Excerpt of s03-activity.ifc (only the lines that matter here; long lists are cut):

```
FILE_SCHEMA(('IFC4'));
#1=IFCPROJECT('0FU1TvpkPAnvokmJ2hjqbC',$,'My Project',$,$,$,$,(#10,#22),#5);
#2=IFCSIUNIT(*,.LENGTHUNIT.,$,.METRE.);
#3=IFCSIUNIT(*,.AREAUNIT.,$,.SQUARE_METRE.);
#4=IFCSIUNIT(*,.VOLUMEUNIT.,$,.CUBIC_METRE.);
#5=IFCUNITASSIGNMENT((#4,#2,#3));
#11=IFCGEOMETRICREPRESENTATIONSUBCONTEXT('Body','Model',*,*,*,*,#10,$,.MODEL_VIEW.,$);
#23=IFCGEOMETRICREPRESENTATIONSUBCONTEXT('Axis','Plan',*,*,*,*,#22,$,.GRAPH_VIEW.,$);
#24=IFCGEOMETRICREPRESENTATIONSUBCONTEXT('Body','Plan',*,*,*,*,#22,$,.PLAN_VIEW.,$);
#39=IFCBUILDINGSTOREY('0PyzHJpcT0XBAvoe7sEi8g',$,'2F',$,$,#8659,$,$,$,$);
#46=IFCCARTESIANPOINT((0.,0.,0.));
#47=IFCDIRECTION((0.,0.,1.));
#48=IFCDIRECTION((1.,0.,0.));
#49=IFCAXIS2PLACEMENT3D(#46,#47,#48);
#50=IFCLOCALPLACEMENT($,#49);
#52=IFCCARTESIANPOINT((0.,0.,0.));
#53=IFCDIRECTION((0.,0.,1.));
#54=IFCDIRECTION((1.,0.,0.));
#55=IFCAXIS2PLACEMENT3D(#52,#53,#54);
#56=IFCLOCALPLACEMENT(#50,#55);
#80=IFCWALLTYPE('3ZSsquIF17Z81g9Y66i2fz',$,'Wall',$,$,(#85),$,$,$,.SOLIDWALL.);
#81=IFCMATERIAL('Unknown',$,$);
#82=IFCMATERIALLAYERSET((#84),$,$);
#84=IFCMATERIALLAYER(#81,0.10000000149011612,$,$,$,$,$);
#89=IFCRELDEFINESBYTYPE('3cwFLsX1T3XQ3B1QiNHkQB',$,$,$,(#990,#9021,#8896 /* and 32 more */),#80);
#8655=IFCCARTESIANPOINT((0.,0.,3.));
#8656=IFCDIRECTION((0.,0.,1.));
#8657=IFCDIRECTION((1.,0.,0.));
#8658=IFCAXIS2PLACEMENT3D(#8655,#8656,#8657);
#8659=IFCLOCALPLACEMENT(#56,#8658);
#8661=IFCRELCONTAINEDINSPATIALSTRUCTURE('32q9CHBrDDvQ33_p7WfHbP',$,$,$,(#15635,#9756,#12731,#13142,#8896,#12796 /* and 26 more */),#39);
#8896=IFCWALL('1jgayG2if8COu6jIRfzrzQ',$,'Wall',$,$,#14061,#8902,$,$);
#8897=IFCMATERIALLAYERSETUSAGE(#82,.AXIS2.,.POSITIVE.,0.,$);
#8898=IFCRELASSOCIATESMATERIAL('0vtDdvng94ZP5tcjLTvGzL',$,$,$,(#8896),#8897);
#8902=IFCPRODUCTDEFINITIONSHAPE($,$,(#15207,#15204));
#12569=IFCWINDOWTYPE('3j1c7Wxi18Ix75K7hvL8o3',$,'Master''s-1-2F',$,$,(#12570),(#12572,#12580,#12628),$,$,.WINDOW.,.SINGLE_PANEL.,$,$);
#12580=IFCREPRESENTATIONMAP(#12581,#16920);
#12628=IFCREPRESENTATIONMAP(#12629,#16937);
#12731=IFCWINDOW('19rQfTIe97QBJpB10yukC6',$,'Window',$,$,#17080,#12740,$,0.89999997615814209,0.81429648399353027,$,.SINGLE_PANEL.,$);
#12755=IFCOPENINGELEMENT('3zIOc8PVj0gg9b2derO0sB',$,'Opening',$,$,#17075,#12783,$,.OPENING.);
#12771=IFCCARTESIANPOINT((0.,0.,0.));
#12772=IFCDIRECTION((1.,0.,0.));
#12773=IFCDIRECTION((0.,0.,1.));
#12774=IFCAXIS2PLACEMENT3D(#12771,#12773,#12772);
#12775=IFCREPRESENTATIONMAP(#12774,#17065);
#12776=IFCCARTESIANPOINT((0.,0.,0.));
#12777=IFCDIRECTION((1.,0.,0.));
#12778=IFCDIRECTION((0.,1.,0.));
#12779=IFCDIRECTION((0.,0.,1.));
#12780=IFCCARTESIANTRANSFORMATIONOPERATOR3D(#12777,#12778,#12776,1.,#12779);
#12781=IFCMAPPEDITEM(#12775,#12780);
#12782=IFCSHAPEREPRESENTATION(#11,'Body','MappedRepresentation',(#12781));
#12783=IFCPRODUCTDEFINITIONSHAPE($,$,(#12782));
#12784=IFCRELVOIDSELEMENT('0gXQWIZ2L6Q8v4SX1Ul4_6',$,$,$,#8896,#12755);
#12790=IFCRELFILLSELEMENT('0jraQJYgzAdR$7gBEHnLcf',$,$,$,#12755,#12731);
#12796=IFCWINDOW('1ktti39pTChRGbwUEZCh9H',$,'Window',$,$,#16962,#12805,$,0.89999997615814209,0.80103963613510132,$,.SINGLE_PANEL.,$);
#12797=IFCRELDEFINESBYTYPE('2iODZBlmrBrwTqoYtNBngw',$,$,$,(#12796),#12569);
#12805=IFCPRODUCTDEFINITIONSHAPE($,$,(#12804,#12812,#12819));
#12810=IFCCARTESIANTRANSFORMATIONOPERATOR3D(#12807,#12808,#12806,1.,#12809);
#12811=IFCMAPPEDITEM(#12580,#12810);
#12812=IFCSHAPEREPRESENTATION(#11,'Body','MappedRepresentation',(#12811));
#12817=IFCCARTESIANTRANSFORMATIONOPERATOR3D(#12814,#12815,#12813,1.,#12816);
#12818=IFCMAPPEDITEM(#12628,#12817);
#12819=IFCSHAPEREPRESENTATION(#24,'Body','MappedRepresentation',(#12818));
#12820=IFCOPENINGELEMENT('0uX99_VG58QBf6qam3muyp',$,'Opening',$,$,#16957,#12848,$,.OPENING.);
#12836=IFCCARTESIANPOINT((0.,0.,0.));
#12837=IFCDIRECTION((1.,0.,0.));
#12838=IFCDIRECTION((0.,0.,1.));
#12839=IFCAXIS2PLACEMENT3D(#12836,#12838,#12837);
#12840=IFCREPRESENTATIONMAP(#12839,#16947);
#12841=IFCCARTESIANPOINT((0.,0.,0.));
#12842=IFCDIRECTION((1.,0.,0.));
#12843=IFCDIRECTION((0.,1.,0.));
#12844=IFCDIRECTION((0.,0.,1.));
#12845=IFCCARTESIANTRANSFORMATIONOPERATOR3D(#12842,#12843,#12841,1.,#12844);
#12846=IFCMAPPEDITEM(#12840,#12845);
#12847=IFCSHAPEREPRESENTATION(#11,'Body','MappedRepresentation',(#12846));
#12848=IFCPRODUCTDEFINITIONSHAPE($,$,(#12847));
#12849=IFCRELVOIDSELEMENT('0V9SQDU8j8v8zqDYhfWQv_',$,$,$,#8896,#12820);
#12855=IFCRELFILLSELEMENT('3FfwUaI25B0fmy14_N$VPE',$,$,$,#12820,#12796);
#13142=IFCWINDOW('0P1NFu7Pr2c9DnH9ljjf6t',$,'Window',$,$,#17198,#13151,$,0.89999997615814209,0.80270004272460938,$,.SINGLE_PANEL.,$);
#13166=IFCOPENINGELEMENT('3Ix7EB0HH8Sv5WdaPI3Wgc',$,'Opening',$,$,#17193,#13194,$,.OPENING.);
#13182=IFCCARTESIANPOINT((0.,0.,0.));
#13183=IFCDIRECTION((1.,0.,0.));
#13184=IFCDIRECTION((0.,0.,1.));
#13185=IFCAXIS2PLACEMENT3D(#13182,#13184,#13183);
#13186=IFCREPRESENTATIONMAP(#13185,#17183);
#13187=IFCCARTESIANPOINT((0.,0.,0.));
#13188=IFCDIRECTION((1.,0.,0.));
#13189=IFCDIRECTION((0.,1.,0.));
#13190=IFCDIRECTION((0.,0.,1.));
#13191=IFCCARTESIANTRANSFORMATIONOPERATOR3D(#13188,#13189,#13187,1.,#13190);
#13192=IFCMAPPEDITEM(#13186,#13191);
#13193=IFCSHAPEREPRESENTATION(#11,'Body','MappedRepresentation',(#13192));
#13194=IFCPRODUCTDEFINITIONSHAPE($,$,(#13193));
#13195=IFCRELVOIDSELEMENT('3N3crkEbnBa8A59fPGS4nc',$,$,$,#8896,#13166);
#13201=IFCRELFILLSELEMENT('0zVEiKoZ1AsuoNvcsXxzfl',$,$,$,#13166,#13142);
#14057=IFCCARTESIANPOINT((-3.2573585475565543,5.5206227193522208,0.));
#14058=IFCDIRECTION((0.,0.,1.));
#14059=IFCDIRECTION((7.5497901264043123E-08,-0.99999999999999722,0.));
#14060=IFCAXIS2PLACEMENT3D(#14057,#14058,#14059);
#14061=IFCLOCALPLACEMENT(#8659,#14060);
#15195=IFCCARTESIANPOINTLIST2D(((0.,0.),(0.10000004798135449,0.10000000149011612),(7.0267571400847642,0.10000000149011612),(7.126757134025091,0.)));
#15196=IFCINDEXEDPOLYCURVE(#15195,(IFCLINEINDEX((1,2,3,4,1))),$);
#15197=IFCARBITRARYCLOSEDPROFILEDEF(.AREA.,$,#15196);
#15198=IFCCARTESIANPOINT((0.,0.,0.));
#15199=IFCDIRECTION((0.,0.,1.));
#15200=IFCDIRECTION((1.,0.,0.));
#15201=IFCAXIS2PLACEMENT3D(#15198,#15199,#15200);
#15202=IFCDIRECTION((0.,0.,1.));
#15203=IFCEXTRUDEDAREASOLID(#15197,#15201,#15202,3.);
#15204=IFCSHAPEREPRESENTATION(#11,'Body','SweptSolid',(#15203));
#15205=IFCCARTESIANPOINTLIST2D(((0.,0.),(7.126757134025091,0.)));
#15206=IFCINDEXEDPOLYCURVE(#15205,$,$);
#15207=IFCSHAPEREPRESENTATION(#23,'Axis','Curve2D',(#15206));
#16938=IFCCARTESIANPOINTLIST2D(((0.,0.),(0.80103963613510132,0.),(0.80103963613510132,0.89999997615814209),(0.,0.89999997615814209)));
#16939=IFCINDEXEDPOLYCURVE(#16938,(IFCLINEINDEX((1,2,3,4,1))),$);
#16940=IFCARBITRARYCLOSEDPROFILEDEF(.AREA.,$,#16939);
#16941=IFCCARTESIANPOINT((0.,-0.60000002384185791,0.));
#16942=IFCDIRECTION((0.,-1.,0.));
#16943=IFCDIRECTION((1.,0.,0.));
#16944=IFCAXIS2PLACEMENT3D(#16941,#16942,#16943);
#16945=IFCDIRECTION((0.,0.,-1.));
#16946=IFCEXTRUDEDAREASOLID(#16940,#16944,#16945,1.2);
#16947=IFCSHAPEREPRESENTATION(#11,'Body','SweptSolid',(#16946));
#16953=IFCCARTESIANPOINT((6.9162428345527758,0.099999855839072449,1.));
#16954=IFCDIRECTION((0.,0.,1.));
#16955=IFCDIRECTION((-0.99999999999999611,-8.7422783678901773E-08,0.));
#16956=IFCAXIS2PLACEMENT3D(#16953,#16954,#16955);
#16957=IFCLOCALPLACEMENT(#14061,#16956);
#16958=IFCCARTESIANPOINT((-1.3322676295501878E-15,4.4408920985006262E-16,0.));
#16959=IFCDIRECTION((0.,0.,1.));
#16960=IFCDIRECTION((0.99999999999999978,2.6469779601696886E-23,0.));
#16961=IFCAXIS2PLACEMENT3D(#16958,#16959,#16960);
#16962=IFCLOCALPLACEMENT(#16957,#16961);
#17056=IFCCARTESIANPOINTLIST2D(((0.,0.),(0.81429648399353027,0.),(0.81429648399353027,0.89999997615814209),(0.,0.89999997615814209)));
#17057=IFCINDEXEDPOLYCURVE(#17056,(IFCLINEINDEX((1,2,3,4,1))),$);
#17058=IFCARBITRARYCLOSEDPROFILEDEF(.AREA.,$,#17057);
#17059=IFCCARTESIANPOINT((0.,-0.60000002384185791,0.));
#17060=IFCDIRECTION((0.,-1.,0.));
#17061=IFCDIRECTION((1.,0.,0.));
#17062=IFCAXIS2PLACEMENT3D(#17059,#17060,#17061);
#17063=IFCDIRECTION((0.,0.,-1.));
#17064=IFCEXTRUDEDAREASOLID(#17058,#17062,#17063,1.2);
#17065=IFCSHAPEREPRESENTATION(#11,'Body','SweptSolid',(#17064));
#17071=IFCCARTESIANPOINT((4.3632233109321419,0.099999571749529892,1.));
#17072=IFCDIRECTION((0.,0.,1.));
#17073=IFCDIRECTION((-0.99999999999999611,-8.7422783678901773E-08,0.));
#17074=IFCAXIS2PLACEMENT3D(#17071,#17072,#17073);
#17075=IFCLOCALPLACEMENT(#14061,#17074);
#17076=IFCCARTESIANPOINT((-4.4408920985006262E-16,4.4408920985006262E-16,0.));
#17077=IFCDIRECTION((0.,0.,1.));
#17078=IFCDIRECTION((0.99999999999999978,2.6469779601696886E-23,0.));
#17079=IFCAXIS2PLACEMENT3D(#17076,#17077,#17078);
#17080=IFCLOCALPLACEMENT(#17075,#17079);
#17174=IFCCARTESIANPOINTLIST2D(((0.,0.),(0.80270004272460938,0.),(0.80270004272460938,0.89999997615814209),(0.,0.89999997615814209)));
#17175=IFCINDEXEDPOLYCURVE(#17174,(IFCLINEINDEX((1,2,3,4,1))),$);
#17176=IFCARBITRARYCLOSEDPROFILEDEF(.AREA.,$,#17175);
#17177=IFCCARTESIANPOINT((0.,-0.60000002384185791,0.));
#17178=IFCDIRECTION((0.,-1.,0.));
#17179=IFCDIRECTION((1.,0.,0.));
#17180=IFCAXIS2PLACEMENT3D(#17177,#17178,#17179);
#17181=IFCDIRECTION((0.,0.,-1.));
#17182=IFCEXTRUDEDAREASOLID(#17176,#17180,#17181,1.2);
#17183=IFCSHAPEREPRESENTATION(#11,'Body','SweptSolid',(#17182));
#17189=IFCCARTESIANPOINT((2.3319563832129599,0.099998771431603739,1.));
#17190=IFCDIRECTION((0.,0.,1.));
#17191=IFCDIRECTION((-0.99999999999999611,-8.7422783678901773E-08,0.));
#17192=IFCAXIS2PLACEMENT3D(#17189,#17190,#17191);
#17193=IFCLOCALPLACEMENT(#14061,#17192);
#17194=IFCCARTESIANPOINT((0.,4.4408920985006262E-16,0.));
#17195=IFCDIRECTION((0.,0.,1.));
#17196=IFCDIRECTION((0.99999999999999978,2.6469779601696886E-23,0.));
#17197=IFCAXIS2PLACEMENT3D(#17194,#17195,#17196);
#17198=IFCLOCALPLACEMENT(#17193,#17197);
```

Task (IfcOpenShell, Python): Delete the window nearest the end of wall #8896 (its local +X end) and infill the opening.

```python
import ifcopenshell
import ifcopenshell.api.feature
import ifcopenshell.api.root
import ifcopenshell.geom
import ifcopenshell.util.shape

model = ifcopenshell.open("s03-activity.ifc")
settings = ifcopenshell.geom.settings()


def volume(element):
    """Net volume in cubic metres, openings subtracted."""
    shape = ifcopenshell.geom.create_shape(settings, element)
    return ifcopenshell.util.shape.get_volume(shape.geometry)


window = model.by_guid("1ktti39pTChRGbwUEZCh9H")
opening = window.FillsVoids[0].RelatingOpeningElement
wall = opening.VoidsElements[0].RelatingBuildingElement
before = volume(wall)

ifcopenshell.api.root.remove_product(model, product=window)
ifcopenshell.api.feature.remove_feature(model, feature=opening)

after = volume(wall)

print(f"wall volume {before:.3f} -> {after:.3f} m3")

model.write("s03-activity_rev.ifc")
```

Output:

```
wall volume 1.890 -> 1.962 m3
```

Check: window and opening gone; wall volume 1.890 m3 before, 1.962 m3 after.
